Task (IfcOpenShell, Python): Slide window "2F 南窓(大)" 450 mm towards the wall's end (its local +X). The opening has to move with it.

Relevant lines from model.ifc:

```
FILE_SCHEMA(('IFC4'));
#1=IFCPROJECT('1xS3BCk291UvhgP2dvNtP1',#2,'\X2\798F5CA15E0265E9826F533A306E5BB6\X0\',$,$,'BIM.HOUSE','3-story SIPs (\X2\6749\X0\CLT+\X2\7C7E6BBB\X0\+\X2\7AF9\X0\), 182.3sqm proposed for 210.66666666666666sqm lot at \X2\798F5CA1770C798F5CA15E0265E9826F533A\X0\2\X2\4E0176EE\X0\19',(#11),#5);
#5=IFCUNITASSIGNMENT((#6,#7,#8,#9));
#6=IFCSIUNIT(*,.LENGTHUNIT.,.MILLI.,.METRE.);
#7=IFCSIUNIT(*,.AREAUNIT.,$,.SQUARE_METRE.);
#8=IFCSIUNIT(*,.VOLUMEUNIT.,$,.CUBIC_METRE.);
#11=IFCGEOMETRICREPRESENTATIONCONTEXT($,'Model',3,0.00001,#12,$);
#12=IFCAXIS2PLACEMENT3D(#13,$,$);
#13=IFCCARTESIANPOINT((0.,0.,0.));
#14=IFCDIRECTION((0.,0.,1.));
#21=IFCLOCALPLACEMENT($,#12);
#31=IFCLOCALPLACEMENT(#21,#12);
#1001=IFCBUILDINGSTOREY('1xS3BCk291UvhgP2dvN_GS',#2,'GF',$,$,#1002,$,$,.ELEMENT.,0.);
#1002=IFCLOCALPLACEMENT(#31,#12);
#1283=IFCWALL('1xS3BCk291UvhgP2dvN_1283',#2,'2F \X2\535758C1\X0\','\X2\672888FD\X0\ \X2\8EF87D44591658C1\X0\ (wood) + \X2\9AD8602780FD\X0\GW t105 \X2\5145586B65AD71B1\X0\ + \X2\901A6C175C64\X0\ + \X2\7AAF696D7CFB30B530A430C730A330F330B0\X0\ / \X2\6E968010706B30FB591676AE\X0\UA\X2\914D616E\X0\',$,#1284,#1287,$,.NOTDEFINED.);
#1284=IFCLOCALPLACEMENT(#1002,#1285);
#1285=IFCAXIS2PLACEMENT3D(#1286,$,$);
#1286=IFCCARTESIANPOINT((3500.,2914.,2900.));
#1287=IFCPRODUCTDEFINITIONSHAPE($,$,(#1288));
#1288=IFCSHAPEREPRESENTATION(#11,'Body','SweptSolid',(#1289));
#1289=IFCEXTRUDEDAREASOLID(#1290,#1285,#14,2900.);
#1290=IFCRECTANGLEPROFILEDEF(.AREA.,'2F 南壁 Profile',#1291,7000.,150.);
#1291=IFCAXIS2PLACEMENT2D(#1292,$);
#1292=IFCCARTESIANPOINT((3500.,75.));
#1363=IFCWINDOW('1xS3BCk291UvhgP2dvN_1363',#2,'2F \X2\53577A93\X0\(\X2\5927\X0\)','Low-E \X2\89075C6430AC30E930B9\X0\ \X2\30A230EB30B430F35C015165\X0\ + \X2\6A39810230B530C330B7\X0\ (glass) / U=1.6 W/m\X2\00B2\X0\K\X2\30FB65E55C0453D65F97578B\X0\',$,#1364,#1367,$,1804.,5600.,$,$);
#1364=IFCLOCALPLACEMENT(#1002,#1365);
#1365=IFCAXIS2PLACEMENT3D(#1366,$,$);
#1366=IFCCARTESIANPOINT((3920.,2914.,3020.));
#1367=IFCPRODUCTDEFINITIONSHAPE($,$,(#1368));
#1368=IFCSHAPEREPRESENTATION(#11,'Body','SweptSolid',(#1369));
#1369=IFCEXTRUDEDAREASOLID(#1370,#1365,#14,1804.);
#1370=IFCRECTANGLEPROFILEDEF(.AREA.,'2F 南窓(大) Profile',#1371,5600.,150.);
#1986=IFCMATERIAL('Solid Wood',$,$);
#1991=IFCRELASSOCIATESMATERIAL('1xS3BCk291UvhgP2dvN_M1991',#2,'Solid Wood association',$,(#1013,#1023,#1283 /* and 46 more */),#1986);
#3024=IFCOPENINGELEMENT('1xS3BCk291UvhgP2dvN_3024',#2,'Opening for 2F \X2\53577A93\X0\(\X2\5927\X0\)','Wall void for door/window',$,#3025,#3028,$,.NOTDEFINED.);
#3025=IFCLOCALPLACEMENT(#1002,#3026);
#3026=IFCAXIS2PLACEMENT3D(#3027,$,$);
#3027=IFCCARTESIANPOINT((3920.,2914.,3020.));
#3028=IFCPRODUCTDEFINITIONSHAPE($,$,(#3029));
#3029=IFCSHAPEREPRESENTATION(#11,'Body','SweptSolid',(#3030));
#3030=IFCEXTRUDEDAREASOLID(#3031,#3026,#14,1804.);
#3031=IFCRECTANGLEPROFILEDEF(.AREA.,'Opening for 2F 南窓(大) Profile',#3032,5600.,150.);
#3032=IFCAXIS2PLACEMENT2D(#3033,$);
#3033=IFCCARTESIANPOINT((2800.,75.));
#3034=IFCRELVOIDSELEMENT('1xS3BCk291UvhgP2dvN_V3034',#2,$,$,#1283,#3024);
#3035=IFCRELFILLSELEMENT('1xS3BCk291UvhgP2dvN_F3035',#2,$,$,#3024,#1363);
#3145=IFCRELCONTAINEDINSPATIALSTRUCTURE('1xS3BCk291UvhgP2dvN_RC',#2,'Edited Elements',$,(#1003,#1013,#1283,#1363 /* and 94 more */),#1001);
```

```python
import ifcopenshell
import ifcopenshell.api.geometry
import ifcopenshell.util.placement

model = ifcopenshell.open("model.ifc")

window = model.by_id(1363)
opening = window.FillsVoids[0].RelatingOpeningElement
wall = opening.VoidsElements[0].RelatingBuildingElement

wall_matrix = ifcopenshell.util.placement.get_local_placement(wall.ObjectPlacement)
shift = wall_matrix[:3, 0] * 450.0
before = ifcopenshell.util.placement.get_local_placement(window.ObjectPlacement)[:3, 3].copy()

# The window is not placed relative to its opening, so move both.
for product in (opening, window):
    matrix = ifcopenshell.util.placement.get_local_placement(product.ObjectPlacement)
    matrix[:3, 3] += shift
    ifcopenshell.api.geometry.edit_object_placement(model, product=product, matrix=matrix, is_si=False)

after = ifcopenshell.util.placement.get_local_placement(window.ObjectPlacement)[:3, 3]
print("window moved by", (after - before).round(3) + 0.0)

model.write("model_updated.ifc")
```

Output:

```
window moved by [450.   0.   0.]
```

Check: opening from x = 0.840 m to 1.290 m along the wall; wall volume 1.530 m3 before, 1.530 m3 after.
